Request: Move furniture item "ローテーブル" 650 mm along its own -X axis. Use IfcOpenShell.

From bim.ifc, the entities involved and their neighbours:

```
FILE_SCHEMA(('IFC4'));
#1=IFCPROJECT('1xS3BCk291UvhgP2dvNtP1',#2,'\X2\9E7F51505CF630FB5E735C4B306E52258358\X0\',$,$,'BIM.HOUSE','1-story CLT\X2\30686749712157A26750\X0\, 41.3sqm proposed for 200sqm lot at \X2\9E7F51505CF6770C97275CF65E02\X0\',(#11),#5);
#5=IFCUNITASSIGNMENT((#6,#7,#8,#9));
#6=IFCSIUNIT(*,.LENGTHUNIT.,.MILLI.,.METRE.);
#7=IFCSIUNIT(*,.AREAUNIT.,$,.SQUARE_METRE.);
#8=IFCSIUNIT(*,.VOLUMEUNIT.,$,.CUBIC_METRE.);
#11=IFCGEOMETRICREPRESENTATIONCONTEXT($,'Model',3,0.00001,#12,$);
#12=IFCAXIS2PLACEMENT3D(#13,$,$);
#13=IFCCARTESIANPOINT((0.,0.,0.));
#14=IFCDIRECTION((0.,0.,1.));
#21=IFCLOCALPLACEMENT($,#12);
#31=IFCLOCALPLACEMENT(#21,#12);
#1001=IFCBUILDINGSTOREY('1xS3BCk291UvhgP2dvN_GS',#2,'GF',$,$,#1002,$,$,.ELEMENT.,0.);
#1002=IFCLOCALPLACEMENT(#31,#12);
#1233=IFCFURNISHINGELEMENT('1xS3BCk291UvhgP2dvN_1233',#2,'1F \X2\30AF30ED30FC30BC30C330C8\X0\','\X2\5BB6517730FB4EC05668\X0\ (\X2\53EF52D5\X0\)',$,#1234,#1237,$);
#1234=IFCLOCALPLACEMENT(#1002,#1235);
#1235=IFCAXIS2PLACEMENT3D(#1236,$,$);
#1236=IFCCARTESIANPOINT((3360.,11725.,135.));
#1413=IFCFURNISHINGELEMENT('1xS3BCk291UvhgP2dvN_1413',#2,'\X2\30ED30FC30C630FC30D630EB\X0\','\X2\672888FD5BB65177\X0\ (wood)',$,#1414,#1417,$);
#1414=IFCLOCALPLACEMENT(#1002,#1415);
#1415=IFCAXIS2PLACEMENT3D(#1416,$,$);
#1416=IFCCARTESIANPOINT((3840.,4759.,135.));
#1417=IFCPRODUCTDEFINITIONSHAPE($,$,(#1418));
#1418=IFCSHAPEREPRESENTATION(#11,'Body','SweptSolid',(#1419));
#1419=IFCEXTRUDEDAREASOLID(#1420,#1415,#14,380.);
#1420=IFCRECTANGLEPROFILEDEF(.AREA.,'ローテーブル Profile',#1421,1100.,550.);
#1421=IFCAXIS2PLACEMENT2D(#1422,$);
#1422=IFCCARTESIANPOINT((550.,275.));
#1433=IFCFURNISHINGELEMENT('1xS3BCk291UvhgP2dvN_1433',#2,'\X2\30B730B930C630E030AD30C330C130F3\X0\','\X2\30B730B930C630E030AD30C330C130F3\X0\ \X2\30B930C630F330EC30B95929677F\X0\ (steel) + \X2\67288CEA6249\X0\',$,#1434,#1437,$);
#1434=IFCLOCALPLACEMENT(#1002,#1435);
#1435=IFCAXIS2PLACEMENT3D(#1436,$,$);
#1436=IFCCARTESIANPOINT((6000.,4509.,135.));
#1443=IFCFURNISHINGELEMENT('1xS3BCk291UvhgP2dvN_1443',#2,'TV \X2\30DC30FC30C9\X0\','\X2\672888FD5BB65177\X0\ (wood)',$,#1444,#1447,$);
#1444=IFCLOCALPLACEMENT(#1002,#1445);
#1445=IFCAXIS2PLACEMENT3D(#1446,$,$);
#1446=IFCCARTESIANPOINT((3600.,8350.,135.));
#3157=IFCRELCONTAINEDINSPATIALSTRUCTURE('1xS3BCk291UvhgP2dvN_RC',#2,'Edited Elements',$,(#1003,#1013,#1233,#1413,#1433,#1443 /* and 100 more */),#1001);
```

```python
import ifcopenshell
import ifcopenshell.api.geometry
import ifcopenshell.util.placement
import ifcopenshell.util.unit

model = ifcopenshell.open("bim.ifc")
unit_scale = ifcopenshell.util.unit.calculate_unit_scale(model)

item = model.by_guid("1xS3BCk291UvhgP2dvN_1413")
matrix = ifcopenshell.util.placement.get_local_placement(item.ObjectPlacement)
matrix[:3, 3] -= matrix[:3, 0] * 0.65 / unit_scale
ifcopenshell.api.geometry.edit_object_placement(model, product=item, matrix=matrix, is_si=False)

print(ifcopenshell.util.placement.get_local_placement(item.ObjectPlacement).round(3) + 0.0)

model.write("bim_updated.ifc")
```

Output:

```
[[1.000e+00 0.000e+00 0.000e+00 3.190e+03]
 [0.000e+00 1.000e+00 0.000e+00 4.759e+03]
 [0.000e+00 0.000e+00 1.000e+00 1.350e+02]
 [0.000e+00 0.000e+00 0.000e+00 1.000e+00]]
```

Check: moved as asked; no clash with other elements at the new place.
